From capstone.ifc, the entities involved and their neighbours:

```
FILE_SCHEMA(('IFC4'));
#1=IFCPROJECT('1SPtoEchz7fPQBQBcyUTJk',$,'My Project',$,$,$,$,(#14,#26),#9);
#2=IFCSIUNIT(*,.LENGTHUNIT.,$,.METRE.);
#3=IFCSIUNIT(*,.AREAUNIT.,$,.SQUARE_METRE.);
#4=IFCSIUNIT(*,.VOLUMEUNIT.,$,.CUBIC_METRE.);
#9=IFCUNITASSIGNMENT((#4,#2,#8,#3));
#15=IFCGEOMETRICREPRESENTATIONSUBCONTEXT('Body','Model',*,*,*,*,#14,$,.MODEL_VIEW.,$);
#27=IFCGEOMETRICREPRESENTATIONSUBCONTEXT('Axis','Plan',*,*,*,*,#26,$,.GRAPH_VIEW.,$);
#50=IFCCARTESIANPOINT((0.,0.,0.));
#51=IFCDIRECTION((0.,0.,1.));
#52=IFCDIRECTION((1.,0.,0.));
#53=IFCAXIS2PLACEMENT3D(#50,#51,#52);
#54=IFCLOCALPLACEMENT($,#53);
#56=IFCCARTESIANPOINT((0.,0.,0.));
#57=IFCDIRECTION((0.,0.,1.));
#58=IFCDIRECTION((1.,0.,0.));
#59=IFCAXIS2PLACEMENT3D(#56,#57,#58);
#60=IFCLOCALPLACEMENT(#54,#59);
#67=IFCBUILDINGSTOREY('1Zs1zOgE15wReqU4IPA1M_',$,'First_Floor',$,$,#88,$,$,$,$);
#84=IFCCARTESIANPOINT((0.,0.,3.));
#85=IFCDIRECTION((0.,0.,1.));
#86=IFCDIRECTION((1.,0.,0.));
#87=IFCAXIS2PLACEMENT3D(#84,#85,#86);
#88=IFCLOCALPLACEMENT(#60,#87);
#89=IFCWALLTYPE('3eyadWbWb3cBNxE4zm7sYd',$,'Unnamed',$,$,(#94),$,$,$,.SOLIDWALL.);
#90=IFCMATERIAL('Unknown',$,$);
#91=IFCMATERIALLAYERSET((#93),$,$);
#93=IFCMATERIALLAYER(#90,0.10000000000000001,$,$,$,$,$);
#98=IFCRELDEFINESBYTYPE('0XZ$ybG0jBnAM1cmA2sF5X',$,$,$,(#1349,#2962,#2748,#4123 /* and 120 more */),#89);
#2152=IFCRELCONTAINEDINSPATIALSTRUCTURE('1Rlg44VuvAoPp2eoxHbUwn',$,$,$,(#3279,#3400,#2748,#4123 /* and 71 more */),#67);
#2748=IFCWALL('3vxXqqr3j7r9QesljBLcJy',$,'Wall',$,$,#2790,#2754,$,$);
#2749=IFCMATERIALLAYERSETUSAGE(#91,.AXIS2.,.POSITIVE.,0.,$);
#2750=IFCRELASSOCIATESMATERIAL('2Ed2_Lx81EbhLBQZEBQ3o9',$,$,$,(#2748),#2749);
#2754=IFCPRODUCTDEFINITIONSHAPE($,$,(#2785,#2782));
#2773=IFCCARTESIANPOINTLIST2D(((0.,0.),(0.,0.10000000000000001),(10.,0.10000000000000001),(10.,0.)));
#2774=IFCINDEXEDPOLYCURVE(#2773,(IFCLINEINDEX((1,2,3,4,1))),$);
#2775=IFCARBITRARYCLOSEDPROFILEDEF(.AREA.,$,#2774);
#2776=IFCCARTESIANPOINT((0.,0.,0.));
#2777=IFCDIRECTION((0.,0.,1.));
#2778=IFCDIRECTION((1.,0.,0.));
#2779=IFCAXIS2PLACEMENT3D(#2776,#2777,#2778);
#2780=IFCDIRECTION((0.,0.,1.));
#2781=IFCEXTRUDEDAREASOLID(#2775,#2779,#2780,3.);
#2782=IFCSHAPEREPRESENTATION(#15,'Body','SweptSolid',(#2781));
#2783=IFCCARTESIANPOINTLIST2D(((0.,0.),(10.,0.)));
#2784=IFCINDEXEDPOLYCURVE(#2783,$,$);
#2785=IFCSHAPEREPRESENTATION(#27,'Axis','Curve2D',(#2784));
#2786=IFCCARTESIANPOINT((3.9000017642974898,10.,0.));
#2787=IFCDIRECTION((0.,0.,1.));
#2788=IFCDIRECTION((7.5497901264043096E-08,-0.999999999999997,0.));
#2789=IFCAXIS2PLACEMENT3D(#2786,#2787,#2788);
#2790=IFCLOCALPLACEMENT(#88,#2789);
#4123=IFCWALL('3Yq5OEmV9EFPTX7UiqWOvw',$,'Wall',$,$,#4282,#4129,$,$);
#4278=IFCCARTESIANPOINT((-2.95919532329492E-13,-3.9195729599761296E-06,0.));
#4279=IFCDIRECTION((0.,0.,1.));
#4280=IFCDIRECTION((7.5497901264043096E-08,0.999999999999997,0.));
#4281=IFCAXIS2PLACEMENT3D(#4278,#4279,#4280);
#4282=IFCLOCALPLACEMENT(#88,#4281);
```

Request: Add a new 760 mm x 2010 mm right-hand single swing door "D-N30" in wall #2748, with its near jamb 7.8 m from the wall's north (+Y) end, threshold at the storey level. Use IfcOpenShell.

```python
import numpy as np
import ifcopenshell
import ifcopenshell.api.feature
import ifcopenshell.api.geometry
import ifcopenshell.api.root
import ifcopenshell.api.spatial
import ifcopenshell.geom
import ifcopenshell.util.element
import ifcopenshell.util.placement
import ifcopenshell.util.representation
import ifcopenshell.util.shape
import ifcopenshell.util.unit

model = ifcopenshell.open("capstone.ifc")
unit_scale = ifcopenshell.util.unit.calculate_unit_scale(model)
settings = ifcopenshell.geom.settings()


def volume(element):
    """Net volume in cubic metres, openings subtracted."""
    shape = ifcopenshell.geom.create_shape(settings, element)
    return ifcopenshell.util.shape.get_volume(shape.geometry)


wall = model.by_guid("3vxXqqr3j7r9QesljBLcJy")
storey = ifcopenshell.util.element.get_container(wall, ifc_class="IfcBuildingStorey")
context = ifcopenshell.util.representation.get_context(model, "Model", "Body", "MODEL_VIEW")
before = volume(wall)

width, height, from_end, sill = 0.76, 2.01, 7.8, 0.0  # metres

# The wall runs along its own X axis, and the end named is its -X end.
wall_shape = ifcopenshell.geom.create_shape(settings, wall)
x, y, z = ifcopenshell.util.shape.get_vertices(wall_shape.geometry).T
start = x.min() + from_end
face, thickness = float(y.min()), float(y.max() - y.min())
wall_matrix = ifcopenshell.util.placement.get_local_placement(wall.ObjectPlacement)
level = ifcopenshell.util.placement.get_local_placement(storey.ObjectPlacement)[2, 3]


def in_wall(x, y):
    """Placement at x, y metres in the wall's axes, at sill height."""
    matrix = wall_matrix.copy()
    matrix[:, 3] = wall_matrix @ np.array([x / unit_scale, y / unit_scale, 0.0, 1.0])
    matrix[2, 3] = level + sill / unit_scale
    return matrix


# Opening: a box that overshoots both wall faces by 50 mm.
opening = ifcopenshell.api.root.create_entity(model, ifc_class="IfcOpeningElement", predefined_type="OPENING")
box = ifcopenshell.api.geometry.add_wall_representation(
    model, context=context, length=width, height=height, thickness=thickness + 0.1
)
ifcopenshell.api.geometry.assign_representation(model, product=opening, representation=box)
ifcopenshell.api.geometry.edit_object_placement(model, product=opening, matrix=in_wall(start, face - 0.05), is_si=False)
ifcopenshell.api.feature.add_feature(model, feature=opening, element=wall)

door = ifcopenshell.api.root.create_entity(model, ifc_class="IfcDoor", name="D-N30", predefined_type="DOOR")
door.OverallWidth, door.OverallHeight = width / unit_scale, height / unit_scale
door.OperationType = "SINGLE_SWING_RIGHT"
body = ifcopenshell.api.geometry.add_door_representation(
    model,
    context=context,
    overall_width=door.OverallWidth,
    overall_height=door.OverallHeight,
    operation_type="SINGLE_SWING_RIGHT",
    lining_properties={"LiningDepth": thickness / unit_scale, "ThresholdDepth": thickness / unit_scale},
)
ifcopenshell.api.geometry.assign_representation(model, product=door, representation=body)
ifcopenshell.api.spatial.assign_container(model, products=[door], relating_structure=storey)
ifcopenshell.api.feature.add_filling(model, opening=opening, element=door)

# The lining spans the wall, so the door starts at the wall face.
ifcopenshell.api.geometry.edit_object_placement(model, product=door, matrix=in_wall(start, face), is_si=False)

after = volume(wall)

print(f"wall volume {before:.3f} -> {after:.3f} m3")

model.write("capstone_edited.ifc")
```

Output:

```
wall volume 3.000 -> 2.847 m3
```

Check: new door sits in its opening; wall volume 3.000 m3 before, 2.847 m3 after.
